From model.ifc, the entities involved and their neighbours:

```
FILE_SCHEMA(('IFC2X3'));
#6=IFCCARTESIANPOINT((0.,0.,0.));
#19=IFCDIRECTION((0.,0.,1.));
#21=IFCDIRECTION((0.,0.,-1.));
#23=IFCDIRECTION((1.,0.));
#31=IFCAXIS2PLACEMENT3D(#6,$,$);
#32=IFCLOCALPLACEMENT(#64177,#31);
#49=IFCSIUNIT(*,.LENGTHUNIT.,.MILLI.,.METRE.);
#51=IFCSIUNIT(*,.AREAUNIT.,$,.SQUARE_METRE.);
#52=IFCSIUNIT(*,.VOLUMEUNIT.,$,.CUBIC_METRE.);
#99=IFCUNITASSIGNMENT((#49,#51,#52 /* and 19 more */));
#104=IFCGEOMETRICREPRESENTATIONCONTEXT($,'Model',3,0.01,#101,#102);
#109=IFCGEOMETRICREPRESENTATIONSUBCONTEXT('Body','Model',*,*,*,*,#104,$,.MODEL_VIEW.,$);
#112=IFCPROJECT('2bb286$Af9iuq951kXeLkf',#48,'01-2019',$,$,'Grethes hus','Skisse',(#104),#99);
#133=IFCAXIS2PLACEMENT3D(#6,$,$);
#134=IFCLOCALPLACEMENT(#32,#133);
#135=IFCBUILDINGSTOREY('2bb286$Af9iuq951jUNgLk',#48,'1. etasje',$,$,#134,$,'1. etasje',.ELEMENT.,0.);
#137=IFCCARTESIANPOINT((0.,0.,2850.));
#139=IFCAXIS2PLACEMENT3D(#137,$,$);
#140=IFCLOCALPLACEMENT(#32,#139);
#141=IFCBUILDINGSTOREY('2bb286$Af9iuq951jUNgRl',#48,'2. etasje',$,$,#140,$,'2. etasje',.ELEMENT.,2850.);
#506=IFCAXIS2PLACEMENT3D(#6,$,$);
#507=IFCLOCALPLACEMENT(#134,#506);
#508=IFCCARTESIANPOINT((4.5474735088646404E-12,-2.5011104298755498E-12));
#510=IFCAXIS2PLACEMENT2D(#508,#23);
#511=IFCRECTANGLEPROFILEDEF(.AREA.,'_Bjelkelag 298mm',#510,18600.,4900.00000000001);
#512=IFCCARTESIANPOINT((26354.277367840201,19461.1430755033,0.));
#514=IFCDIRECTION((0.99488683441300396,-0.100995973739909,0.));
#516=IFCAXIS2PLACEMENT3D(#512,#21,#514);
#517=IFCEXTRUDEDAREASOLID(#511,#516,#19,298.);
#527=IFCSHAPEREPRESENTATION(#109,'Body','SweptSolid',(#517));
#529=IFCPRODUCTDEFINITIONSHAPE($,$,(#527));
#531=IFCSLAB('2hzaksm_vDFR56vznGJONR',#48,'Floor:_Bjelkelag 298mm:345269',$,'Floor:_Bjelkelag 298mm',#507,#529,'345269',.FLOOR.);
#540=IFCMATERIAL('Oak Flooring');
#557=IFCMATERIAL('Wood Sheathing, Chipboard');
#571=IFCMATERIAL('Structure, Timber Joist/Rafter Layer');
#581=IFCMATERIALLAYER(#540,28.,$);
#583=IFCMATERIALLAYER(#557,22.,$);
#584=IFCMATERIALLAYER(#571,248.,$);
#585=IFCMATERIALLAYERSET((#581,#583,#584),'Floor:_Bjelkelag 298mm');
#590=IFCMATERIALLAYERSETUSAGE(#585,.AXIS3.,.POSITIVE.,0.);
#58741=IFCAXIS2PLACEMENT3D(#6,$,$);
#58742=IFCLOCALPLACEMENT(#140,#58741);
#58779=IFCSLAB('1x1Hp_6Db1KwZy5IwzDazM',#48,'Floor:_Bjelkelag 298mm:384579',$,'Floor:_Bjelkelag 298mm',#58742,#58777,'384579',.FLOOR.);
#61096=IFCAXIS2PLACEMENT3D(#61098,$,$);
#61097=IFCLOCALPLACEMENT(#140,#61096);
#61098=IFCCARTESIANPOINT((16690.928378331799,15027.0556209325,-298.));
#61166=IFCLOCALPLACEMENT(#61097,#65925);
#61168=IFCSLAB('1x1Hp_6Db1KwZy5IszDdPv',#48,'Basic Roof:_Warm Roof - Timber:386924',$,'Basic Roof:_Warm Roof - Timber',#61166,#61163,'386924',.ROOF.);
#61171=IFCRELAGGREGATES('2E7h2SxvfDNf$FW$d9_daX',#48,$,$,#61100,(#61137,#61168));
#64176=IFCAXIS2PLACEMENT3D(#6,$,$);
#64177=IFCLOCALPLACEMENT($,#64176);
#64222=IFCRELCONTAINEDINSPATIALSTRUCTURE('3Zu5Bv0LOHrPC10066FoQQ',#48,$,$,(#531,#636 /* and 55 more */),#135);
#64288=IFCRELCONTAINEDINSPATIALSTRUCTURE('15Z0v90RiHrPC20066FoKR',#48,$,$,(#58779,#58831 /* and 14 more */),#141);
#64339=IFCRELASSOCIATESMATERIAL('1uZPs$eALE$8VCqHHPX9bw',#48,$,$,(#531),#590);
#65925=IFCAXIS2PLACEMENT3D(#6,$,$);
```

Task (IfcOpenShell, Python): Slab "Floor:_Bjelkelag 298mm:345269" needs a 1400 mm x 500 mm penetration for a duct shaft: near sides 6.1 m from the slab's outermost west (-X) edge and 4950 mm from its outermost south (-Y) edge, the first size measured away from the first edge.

```python
import numpy as np
import ifcopenshell
import ifcopenshell.api.feature
import ifcopenshell.api.geometry
import ifcopenshell.api.root
import ifcopenshell.geom
import ifcopenshell.util.placement
import ifcopenshell.util.representation
import ifcopenshell.util.shape
import ifcopenshell.util.unit

model = ifcopenshell.open("model.ifc")
unit_scale = ifcopenshell.util.unit.calculate_unit_scale(model)
settings = ifcopenshell.geom.settings()


def volume(element):
    """Net volume in cubic metres, openings subtracted."""
    shape = ifcopenshell.geom.create_shape(settings, element)
    return ifcopenshell.util.shape.get_volume(shape.geometry)


slab = model.by_id(531)
before = volume(slab)

# Extent in the slab's own axes, in metres. The edges named are its -X and -Y sides.
slab_shape = ifcopenshell.geom.create_shape(settings, slab)
vertices = ifcopenshell.util.shape.get_vertices(slab_shape.geometry)
x_min, y_min, bottom = vertices.min(axis=0)
top = vertices[:, 2].max()

opening = ifcopenshell.api.root.create_entity(model, ifc_class="IfcOpeningElement", name="Duct shaft opening")
context = ifcopenshell.util.representation.get_context(model, "Model", "Body", "MODEL_VIEW")
width, depth = 1.4, 0.5
outline = [(0.0, 0.0), (width, 0.0), (width, depth), (0.0, depth), (0.0, 0.0)]
# Overshoot both faces by 50 mm so the cut is clean.
shape = ifcopenshell.api.geometry.add_slab_representation(
    model, context=context, depth=top - bottom + 0.1, polyline=outline
)
ifcopenshell.api.geometry.assign_representation(model, product=opening, representation=shape)

matrix = ifcopenshell.util.placement.get_local_placement(slab.ObjectPlacement)
matrix[:, 3] = matrix @ np.append(np.array([x_min + 6.1, y_min + 4.95, bottom - 0.05]) / unit_scale, 1.0)
ifcopenshell.api.geometry.edit_object_placement(model, product=opening, matrix=matrix, is_si=False)
ifcopenshell.api.feature.add_feature(model, feature=opening, element=slab)

after = volume(slab)

print(f"slab volume {before:.3f} -> {after:.3f} m3")

model.write("model_v2.ifc")
```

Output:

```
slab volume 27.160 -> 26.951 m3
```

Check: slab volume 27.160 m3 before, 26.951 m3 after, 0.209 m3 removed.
